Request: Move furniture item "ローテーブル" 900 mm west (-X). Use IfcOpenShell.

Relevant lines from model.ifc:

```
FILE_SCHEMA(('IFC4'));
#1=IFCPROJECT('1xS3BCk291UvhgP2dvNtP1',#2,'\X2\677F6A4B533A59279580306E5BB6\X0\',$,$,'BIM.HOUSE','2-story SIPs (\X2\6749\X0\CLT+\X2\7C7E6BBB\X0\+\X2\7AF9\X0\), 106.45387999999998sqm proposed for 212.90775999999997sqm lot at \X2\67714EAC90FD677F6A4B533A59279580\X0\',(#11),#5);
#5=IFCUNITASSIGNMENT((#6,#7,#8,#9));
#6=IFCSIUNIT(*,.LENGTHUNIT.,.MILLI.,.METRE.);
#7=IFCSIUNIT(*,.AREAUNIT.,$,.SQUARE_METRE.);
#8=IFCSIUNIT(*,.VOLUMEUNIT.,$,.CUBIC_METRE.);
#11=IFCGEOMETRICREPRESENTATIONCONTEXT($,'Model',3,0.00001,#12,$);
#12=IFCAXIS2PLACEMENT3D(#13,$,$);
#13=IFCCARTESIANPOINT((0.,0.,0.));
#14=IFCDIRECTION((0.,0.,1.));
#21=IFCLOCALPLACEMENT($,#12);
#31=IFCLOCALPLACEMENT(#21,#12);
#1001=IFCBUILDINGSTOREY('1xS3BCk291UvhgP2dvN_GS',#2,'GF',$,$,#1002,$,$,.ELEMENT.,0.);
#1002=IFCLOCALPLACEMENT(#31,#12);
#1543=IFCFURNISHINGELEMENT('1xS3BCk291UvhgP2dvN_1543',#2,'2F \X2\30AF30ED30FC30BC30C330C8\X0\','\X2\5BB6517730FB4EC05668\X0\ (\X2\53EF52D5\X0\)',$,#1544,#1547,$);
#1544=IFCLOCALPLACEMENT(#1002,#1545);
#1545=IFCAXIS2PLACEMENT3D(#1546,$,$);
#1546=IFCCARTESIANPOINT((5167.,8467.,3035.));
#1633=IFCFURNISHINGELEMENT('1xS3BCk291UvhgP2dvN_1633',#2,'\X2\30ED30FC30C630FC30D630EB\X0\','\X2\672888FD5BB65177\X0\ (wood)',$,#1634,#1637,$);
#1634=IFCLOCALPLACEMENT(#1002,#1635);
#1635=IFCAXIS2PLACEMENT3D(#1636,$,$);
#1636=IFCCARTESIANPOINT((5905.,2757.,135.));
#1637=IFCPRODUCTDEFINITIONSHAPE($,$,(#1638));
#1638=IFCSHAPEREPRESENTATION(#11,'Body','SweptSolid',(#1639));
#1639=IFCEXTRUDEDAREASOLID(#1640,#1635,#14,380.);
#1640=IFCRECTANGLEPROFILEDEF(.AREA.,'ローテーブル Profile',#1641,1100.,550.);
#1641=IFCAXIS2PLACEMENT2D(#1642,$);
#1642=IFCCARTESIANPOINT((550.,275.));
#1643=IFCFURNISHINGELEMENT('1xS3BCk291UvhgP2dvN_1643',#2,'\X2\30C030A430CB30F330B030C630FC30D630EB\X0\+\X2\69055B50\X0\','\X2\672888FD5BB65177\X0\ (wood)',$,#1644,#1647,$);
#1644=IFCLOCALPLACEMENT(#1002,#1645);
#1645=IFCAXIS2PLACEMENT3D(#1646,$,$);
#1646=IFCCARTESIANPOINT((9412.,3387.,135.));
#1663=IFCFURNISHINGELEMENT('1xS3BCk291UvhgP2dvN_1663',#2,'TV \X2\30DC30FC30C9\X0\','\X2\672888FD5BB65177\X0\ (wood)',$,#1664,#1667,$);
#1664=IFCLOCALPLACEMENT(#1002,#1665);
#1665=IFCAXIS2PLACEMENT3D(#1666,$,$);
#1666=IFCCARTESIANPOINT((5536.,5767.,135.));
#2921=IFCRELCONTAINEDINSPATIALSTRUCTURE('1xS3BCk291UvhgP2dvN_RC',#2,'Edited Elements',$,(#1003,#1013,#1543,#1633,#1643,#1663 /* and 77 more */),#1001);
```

```python
import ifcopenshell
import ifcopenshell.api.geometry
import ifcopenshell.util.placement
import ifcopenshell.util.unit

model = ifcopenshell.open("model.ifc")
unit_scale = ifcopenshell.util.unit.calculate_unit_scale(model)

item = model.by_guid("1xS3BCk291UvhgP2dvN_1633")
matrix = ifcopenshell.util.placement.get_local_placement(item.ObjectPlacement)
matrix[0, 3] -= 0.9 / unit_scale
ifcopenshell.api.geometry.edit_object_placement(model, product=item, matrix=matrix, is_si=False)

print(ifcopenshell.util.placement.get_local_placement(item.ObjectPlacement).round(3) + 0.0)

model.write("model_edited.ifc")
```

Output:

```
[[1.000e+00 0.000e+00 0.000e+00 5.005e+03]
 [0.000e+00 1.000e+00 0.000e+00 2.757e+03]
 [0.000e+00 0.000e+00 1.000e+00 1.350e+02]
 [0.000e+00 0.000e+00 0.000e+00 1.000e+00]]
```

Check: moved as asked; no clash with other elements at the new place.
